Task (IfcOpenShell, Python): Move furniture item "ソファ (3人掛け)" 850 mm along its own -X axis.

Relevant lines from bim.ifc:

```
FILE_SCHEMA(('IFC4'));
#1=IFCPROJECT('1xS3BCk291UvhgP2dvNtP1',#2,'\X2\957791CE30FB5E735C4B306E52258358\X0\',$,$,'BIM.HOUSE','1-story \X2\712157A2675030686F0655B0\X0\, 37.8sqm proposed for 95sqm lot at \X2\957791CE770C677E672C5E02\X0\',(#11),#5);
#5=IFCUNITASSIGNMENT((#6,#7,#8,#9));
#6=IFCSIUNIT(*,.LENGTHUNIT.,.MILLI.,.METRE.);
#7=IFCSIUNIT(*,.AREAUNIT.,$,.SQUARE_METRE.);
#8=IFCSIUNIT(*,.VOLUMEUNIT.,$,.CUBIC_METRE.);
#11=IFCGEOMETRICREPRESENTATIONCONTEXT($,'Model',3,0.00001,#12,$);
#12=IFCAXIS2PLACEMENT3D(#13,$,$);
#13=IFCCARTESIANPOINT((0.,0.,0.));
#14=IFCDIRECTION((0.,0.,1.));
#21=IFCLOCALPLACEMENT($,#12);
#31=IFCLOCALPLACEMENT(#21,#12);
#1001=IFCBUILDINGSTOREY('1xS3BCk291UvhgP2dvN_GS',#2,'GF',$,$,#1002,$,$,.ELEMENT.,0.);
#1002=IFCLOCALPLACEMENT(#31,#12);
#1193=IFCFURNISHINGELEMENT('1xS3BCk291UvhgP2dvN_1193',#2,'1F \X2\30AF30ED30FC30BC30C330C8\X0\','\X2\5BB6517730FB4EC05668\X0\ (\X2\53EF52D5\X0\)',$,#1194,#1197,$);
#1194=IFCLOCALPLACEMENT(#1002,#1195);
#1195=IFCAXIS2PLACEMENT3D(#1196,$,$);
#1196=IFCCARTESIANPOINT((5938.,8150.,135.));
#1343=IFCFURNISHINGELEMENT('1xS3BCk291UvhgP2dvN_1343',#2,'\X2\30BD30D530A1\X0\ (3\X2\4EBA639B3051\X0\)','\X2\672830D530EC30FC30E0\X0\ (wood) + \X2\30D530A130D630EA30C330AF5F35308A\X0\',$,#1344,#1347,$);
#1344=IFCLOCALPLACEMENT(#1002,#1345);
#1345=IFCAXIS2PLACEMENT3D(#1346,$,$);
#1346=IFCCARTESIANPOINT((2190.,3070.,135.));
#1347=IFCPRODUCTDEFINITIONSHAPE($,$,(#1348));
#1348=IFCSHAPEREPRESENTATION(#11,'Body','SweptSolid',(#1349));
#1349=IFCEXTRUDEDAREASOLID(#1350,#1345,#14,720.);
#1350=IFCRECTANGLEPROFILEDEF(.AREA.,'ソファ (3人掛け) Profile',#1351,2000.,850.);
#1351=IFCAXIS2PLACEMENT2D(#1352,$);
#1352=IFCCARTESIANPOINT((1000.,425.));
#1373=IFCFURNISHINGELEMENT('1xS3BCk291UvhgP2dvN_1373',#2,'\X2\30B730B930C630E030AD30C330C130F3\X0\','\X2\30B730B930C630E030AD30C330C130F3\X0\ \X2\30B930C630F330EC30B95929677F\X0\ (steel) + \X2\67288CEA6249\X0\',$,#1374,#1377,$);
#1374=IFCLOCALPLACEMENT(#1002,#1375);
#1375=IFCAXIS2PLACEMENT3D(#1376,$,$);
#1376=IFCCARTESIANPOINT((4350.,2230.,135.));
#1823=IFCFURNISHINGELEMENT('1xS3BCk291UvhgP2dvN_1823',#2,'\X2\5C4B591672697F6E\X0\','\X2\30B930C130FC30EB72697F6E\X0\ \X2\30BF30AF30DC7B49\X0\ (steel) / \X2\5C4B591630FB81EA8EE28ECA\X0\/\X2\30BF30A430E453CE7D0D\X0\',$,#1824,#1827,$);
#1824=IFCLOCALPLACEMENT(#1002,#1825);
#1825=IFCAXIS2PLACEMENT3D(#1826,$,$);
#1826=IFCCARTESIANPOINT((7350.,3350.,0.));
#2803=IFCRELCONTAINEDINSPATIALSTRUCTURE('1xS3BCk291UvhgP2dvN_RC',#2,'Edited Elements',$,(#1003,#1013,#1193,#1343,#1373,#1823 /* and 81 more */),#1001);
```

```python
import ifcopenshell
import ifcopenshell.api.geometry
import ifcopenshell.util.placement

model = ifcopenshell.open("bim.ifc")

item = model.by_guid("1xS3BCk291UvhgP2dvN_1343")
matrix = ifcopenshell.util.placement.get_local_placement(item.ObjectPlacement)
matrix[:3, 3] -= matrix[:3, 0] * 850.0
ifcopenshell.api.geometry.edit_object_placement(model, product=item, matrix=matrix, is_si=False)

print(ifcopenshell.util.placement.get_local_placement(item.ObjectPlacement).round(3) + 0.0)

model.write("bim_edited.ifc")
```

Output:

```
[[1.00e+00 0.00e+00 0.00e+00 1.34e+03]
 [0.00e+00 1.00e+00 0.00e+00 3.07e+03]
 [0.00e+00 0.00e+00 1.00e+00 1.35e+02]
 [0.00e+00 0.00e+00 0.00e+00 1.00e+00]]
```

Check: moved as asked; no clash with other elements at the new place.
